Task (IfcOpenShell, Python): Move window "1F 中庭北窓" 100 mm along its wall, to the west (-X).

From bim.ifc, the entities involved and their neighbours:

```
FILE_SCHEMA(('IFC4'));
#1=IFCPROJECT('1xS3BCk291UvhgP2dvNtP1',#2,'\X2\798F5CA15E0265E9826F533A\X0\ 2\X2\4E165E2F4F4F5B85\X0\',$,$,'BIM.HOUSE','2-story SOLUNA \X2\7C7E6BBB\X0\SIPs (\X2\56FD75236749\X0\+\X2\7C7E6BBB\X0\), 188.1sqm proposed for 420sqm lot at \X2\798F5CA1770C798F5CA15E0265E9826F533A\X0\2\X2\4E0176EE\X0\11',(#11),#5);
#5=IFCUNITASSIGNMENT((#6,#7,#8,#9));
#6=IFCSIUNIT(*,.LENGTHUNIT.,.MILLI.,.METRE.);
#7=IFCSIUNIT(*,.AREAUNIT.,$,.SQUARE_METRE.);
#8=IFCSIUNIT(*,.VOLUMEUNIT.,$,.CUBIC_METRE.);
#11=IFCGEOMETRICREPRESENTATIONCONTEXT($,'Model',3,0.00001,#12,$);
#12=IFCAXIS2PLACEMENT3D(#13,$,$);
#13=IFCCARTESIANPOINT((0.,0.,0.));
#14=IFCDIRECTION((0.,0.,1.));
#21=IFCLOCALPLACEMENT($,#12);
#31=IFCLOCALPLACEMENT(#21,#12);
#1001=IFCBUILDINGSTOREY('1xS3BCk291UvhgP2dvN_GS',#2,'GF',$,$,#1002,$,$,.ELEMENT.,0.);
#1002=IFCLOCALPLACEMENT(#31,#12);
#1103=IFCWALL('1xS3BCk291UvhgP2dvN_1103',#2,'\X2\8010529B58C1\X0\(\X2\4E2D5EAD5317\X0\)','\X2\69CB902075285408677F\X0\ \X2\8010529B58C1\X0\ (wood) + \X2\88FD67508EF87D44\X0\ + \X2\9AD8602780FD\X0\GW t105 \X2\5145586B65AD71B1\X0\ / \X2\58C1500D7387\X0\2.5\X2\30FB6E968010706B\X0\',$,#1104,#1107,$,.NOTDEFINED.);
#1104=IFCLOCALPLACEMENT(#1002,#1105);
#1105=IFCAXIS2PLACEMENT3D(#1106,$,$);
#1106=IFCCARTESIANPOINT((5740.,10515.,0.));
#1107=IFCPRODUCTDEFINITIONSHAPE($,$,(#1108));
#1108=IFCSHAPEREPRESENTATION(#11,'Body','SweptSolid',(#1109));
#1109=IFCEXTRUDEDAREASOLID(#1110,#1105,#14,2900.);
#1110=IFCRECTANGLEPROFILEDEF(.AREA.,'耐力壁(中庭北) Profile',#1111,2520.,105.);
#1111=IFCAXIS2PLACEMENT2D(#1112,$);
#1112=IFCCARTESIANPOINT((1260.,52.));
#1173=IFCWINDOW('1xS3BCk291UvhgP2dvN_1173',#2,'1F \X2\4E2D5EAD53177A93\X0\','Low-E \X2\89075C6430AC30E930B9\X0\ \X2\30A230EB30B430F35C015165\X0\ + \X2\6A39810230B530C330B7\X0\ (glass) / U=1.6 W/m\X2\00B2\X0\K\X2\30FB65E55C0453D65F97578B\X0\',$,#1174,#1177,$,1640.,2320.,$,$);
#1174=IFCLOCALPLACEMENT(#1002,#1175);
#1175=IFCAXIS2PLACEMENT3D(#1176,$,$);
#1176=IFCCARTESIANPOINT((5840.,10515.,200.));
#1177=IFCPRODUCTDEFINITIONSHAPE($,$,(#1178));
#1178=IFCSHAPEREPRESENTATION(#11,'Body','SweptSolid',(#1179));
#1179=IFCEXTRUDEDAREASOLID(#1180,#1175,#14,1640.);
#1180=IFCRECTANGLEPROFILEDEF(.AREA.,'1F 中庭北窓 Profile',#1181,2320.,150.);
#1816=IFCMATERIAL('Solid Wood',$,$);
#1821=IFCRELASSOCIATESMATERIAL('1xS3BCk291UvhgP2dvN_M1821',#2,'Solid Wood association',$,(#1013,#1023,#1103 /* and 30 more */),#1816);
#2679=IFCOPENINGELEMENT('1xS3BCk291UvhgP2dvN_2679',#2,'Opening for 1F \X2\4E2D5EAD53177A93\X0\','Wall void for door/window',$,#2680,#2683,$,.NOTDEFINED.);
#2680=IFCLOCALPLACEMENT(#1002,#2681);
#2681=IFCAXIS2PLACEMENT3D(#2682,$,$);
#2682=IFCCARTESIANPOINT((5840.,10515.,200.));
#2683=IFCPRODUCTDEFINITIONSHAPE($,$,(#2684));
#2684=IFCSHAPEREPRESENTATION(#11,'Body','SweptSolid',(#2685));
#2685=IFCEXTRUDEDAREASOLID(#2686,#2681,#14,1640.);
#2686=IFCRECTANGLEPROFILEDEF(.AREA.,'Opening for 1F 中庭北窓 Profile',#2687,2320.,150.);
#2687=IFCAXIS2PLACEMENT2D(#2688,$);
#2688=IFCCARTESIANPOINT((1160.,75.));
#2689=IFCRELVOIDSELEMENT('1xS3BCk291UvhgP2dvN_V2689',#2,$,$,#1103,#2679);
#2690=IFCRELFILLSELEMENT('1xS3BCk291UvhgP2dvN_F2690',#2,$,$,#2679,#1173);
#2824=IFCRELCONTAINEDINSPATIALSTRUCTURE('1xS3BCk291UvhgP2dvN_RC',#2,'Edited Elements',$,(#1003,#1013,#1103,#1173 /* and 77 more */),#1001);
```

```python
import ifcopenshell
import ifcopenshell.api.geometry
import ifcopenshell.util.placement

model = ifcopenshell.open("bim.ifc")

window = model.by_guid("1xS3BCk291UvhgP2dvN_1173")
opening = window.FillsVoids[0].RelatingOpeningElement
wall = opening.VoidsElements[0].RelatingBuildingElement

wall_matrix = ifcopenshell.util.placement.get_local_placement(wall.ObjectPlacement)
shift = wall_matrix[:3, 0] * -100.0
before = ifcopenshell.util.placement.get_local_placement(window.ObjectPlacement)[:3, 3].copy()

# The window is not placed relative to its opening, so move both.
for product in (opening, window):
    matrix = ifcopenshell.util.placement.get_local_placement(product.ObjectPlacement)
    matrix[:3, 3] += shift
    ifcopenshell.api.geometry.edit_object_placement(model, product=product, matrix=matrix, is_si=False)

after = ifcopenshell.util.placement.get_local_placement(window.ObjectPlacement)[:3, 3]
print("window moved by", (after - before).round(3) + 0.0)

model.write("bim_v2.ifc")
```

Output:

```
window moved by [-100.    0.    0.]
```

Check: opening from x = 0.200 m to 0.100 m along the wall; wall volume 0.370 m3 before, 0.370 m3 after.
